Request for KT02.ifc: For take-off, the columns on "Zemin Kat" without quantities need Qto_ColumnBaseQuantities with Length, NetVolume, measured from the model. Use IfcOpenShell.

First a look at what the model holds.

```python
import ifcopenshell
import ifcopenshell.util.element
import ifcopenshell.util.unit

model = ifcopenshell.open("KT02.ifc")
print(model.schema)
for unit_type in ("LENGTHUNIT", "AREAUNIT", "VOLUMEUNIT"):
    print(unit_type, ifcopenshell.util.unit.calculate_unit_scale(model, unit_type))
storey = next(s for s in model.by_type("IfcBuildingStorey") if s.Name == "Zemin Kat")
columns = [e for e in ifcopenshell.util.element.get_decomposition(storey) if e.is_a("IfcColumn")]
for e in sorted(columns, key=lambda e: e.id()):
    print(e.id(), e.is_a(), e.Name, list(ifcopenshell.util.element.get_psets(e, qtos_only=True)), sep=" | ")
```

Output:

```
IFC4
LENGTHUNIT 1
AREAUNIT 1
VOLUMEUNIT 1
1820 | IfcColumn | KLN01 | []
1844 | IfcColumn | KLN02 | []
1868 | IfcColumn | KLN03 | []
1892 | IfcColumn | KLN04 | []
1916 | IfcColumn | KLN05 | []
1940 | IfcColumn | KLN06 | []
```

```python
import ifcopenshell
import ifcopenshell.api.pset
import ifcopenshell.geom
import ifcopenshell.util.element
import ifcopenshell.util.shape
import ifcopenshell.util.unit

model = ifcopenshell.open("KT02.ifc")
unit_scale = ifcopenshell.util.unit.calculate_unit_scale(model)
volume_scale = ifcopenshell.util.unit.calculate_unit_scale(model, "VOLUMEUNIT")
settings = ifcopenshell.geom.settings()

storey = next(s for s in model.by_type("IfcBuildingStorey") if s.Name == "Zemin Kat")
columns = [e for e in ifcopenshell.util.element.get_decomposition(storey) if e.is_a("IfcColumn")]

for e in sorted(columns, key=lambda e: e.id()):
    if ifcopenshell.util.element.get_psets(e, qtos_only=True, should_inherit=False):
        continue
    # Geometry comes back in metres, in the element's own axes.
    shape = ifcopenshell.geom.create_shape(settings, e)
    values = {
        "Length": ifcopenshell.util.shape.get_z(shape.geometry) / unit_scale,
        "NetVolume": ifcopenshell.util.shape.get_volume(shape.geometry) / volume_scale,
    }
    qto = ifcopenshell.api.pset.add_qto(model, product=e, name="Qto_ColumnBaseQuantities")
    ifcopenshell.api.pset.edit_qto(model, qto=qto, properties=values)
    print(e.id(), {k: round(v, 3) for k, v in values.items()})

model.write("KT02-out.ifc")
```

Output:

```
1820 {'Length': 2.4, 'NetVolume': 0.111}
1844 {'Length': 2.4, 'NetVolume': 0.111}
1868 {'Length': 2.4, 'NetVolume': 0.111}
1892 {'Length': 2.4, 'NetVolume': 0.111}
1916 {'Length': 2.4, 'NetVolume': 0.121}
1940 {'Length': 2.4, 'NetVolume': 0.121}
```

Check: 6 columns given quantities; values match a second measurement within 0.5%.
